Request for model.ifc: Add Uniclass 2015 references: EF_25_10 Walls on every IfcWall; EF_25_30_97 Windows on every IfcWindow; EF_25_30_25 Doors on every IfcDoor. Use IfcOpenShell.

First a look at what the model holds.

```python
import ifcopenshell

model = ifcopenshell.open("model.ifc")
print(model.schema)
print("classifications:", [c.Name for c in model.by_type("IfcClassification")])
for ifc_class in ("IfcDoor", "IfcRoof", "IfcStair", "IfcWall", "IfcWindow"):
    print(ifc_class, len(model.by_type(ifc_class)))
```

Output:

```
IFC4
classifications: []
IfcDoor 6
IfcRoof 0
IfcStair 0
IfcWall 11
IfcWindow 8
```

```python
import ifcopenshell
import ifcopenshell.api.classification

model = ifcopenshell.open("model.ifc")

system = ifcopenshell.api.classification.add_classification(model, classification="Uniclass 2015")

codes = {
    "IfcWall": ("EF_25_10", "Walls"),
    "IfcWindow": ("EF_25_30_97", "Windows"),
    "IfcDoor": ("EF_25_30_25", "Doors"),
}
for ifc_class, (code, name) in codes.items():
    products = model.by_type(ifc_class)
    ifcopenshell.api.classification.add_reference(
        model, products=products, classification=system, identification=code, name=name
    )
    print(code, len(products))

model.write("model_edited.ifc")
```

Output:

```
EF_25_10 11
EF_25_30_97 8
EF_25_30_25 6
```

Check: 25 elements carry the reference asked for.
